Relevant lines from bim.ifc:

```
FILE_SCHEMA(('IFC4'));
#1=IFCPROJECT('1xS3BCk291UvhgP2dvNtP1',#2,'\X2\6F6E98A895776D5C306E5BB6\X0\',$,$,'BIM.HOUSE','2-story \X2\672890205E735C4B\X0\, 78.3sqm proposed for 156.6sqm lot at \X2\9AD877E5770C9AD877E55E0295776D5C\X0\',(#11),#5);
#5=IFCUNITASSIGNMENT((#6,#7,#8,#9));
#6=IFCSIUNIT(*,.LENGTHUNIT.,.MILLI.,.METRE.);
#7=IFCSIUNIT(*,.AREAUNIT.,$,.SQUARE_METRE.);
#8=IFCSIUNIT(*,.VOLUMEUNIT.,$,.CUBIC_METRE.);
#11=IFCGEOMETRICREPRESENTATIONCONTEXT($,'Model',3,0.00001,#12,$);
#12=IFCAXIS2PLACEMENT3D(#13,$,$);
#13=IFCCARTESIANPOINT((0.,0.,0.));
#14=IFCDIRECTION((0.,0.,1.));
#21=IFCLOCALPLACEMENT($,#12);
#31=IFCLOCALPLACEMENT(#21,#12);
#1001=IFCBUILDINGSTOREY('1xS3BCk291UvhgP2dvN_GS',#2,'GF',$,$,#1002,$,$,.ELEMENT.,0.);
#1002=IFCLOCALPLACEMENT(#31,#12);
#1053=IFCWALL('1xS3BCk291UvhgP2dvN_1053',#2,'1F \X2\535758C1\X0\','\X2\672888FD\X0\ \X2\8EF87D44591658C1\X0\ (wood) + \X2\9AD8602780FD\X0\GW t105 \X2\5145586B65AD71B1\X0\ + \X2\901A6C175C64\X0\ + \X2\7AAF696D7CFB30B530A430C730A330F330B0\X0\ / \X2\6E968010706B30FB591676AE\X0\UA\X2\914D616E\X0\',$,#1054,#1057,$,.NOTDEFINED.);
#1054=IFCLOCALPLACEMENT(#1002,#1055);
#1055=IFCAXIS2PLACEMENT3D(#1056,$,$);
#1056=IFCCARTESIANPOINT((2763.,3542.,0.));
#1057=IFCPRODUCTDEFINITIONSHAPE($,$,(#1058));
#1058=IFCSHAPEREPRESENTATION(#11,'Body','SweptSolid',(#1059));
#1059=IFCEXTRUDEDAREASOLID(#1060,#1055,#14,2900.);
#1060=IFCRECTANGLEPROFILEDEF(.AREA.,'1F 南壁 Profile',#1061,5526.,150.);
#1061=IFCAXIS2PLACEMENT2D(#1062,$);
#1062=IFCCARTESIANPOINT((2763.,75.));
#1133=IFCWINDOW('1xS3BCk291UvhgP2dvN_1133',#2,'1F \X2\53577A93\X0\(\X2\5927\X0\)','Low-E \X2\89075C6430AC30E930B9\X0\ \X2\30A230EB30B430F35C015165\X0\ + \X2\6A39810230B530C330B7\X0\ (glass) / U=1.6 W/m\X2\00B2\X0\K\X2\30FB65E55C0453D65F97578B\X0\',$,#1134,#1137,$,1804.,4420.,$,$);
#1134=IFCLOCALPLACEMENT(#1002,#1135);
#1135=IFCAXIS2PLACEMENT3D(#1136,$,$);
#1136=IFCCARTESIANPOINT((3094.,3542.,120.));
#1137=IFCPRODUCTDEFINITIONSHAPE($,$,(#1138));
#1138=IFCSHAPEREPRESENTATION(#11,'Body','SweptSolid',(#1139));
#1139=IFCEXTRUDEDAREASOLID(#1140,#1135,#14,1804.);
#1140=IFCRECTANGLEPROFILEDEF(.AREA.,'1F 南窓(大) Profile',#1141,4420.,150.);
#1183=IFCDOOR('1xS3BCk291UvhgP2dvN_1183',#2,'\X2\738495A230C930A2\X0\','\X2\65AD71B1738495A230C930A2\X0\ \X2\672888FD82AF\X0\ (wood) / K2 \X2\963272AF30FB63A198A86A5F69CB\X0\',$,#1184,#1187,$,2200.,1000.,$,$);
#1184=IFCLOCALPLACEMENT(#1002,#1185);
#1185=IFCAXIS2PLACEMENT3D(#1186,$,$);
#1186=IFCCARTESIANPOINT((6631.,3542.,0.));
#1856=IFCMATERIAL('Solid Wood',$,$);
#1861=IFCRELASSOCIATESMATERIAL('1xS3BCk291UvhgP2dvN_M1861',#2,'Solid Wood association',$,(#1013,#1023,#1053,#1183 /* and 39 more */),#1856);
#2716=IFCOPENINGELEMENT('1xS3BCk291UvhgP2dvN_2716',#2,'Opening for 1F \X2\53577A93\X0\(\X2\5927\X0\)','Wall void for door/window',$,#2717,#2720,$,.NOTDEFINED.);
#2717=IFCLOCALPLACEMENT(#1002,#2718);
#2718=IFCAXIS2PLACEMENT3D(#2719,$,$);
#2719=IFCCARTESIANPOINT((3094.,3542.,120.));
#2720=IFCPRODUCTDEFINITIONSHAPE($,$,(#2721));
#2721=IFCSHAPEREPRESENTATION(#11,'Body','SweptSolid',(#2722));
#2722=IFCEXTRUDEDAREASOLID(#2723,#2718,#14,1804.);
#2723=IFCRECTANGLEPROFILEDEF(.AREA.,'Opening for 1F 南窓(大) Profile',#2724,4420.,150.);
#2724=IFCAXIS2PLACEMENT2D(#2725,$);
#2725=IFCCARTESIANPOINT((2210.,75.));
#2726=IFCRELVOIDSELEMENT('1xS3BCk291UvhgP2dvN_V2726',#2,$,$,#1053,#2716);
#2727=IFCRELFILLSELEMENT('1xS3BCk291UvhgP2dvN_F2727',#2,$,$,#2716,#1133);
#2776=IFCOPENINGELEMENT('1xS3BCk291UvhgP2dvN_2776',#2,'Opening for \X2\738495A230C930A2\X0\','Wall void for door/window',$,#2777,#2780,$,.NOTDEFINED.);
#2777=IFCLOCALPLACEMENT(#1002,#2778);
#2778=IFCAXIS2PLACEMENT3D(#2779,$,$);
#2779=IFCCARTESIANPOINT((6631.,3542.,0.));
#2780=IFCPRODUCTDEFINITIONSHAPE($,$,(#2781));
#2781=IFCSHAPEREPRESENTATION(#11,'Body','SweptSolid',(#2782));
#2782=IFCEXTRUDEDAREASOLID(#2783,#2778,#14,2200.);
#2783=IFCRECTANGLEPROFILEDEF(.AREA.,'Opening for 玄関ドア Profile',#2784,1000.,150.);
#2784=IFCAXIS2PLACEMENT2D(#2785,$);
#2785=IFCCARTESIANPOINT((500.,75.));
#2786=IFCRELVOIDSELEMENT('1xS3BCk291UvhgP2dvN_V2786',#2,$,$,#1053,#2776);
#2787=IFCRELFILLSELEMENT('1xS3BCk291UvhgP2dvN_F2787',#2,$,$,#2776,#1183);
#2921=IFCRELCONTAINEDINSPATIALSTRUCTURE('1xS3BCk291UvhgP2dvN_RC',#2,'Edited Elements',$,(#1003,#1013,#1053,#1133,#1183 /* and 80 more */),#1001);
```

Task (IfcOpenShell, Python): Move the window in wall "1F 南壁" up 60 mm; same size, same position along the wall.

```python
import numpy as np
import ifcopenshell
import ifcopenshell.api.geometry
import ifcopenshell.util.placement
import ifcopenshell.util.unit

model = ifcopenshell.open("bim.ifc")
unit_scale = ifcopenshell.util.unit.calculate_unit_scale(model)

window = model.by_guid("1xS3BCk291UvhgP2dvN_1133")
opening = window.FillsVoids[0].RelatingOpeningElement
dz = 0.06 / unit_scale

shift = np.array([0.0, 0.0, dz])
# The window is not placed relative to its opening, so move both.
for product in (opening, window):
    matrix = ifcopenshell.util.placement.get_local_placement(product.ObjectPlacement)
    matrix[:3, 3] += shift
    ifcopenshell.api.geometry.edit_object_placement(model, product=product, matrix=matrix, is_si=False)

print(f"moved by {dz * unit_scale:+.3f} m")

model.write("bim_edited.ifc")
```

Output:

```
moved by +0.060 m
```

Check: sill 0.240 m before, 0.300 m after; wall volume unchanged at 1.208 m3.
